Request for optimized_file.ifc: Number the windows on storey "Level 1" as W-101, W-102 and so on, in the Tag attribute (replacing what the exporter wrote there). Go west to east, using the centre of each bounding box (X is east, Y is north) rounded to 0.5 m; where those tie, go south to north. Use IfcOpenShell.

First a look at what the model holds.

```python
import ifcopenshell
import ifcopenshell.util.element
import ifcopenshell.util.placement

model = ifcopenshell.open("optimized_file.ifc")
print(model.schema)
storey = next(s for s in model.by_type("IfcBuildingStorey") if s.Name == "Level 1")
windows = [e for e in ifcopenshell.util.element.get_decomposition(storey) if e.is_a("IfcWindow")]
for e in sorted(windows, key=lambda e: e.id()):
    origin = ifcopenshell.util.placement.get_local_placement(e.ObjectPlacement)[:3, 3]
    print(e.id(), e.Tag, e.Name, origin.round(2) + 0.0, sep=" | ")
```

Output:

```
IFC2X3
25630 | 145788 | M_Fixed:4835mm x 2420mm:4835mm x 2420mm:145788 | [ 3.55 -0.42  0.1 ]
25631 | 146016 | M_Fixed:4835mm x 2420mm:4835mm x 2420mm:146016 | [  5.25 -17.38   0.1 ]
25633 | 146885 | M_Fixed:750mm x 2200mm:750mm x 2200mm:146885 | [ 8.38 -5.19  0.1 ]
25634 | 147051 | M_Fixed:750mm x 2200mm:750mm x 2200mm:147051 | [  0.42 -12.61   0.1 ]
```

```python
import ifcopenshell
import ifcopenshell.geom
import ifcopenshell.util.element
import ifcopenshell.util.shape

model = ifcopenshell.open("optimized_file.ifc")
settings = ifcopenshell.geom.settings()
settings.set("use-world-coords", True)


def centre(element):
    shape = ifcopenshell.geom.create_shape(settings, element)
    return ifcopenshell.util.shape.get_bbox_centroid(shape.geometry)


storey = next(s for s in model.by_type("IfcBuildingStorey") if s.Name == "Level 1")
windows = [e for e in ifcopenshell.util.element.get_decomposition(storey) if e.is_a("IfcWindow")]

# Insertion points can sit at a corner or the storey origin, so sort by the geometry (in metres).
centres = {e: centre(e) for e in windows}
windows.sort(key=lambda e: (round(centres[e][0] / 0.5), centres[e][1]))

for i, e in enumerate(windows, start=1):
    number = f"W-1{i:02d}"
    e.Tag = number
    print(e.id(), number)

model.write("optimized_file-out.ifc")
```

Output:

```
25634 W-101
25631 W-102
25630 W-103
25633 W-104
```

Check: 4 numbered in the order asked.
